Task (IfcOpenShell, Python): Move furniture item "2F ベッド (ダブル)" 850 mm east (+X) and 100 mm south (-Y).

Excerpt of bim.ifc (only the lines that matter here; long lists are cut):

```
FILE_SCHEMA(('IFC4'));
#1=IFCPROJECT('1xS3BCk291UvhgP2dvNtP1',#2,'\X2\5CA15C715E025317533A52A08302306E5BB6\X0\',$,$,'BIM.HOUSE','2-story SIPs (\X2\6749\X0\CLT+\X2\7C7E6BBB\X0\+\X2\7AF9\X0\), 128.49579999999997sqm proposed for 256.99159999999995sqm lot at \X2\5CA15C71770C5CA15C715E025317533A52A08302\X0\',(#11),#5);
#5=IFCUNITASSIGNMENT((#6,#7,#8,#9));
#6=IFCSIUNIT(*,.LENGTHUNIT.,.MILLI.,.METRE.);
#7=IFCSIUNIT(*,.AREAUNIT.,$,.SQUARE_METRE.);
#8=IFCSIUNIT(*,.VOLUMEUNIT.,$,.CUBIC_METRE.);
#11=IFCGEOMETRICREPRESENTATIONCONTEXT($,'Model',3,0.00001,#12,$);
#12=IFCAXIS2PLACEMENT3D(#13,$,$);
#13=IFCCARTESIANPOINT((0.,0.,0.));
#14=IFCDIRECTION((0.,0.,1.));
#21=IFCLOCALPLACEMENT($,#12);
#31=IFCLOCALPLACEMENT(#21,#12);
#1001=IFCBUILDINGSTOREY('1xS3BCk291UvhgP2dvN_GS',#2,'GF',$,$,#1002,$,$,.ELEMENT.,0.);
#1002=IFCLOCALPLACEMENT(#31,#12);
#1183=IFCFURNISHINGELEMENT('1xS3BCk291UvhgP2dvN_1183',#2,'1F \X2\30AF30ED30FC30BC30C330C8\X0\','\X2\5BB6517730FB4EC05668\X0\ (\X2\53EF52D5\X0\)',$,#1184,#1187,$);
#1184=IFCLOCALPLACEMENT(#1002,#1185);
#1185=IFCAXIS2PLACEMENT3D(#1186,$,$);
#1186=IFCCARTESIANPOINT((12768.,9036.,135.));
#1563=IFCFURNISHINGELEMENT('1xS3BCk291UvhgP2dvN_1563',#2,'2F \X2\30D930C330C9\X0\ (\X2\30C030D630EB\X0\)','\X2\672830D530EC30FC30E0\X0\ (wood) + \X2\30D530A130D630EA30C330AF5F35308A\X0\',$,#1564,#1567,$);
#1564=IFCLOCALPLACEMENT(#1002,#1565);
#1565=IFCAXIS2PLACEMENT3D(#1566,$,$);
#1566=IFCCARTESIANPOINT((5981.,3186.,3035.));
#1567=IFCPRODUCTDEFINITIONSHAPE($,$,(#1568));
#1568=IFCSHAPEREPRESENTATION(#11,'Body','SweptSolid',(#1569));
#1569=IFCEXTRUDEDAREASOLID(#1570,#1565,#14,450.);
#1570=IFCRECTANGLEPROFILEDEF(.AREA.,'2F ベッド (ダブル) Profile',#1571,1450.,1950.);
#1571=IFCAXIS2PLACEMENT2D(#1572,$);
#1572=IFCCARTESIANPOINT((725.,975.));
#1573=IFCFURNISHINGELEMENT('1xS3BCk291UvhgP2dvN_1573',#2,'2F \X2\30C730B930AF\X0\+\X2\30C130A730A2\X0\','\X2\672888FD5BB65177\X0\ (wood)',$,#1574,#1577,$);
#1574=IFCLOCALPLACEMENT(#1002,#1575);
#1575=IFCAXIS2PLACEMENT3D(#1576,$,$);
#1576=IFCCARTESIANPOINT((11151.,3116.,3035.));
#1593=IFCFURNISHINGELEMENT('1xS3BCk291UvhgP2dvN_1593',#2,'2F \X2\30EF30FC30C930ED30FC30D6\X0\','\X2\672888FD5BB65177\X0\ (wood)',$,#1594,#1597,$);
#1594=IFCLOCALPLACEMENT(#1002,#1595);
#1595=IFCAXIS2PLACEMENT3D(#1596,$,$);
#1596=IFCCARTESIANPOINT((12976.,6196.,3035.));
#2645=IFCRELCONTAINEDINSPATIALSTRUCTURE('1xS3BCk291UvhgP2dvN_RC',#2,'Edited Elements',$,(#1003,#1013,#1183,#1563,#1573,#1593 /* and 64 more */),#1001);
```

```python
import ifcopenshell
import ifcopenshell.api.geometry
import ifcopenshell.util.placement
import ifcopenshell.util.unit

model = ifcopenshell.open("bim.ifc")
unit_scale = ifcopenshell.util.unit.calculate_unit_scale(model)

item = model.by_guid("1xS3BCk291UvhgP2dvN_1563")
matrix = ifcopenshell.util.placement.get_local_placement(item.ObjectPlacement)
matrix[0, 3] += 0.85 / unit_scale
matrix[1, 3] -= 0.1 / unit_scale
ifcopenshell.api.geometry.edit_object_placement(model, product=item, matrix=matrix, is_si=False)

print(ifcopenshell.util.placement.get_local_placement(item.ObjectPlacement).round(3) + 0.0)

model.write("bim_edited.ifc")
```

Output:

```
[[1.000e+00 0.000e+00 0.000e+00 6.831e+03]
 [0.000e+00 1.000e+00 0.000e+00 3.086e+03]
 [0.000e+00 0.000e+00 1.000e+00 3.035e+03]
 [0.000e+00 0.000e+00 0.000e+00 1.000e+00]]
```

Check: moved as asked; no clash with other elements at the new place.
